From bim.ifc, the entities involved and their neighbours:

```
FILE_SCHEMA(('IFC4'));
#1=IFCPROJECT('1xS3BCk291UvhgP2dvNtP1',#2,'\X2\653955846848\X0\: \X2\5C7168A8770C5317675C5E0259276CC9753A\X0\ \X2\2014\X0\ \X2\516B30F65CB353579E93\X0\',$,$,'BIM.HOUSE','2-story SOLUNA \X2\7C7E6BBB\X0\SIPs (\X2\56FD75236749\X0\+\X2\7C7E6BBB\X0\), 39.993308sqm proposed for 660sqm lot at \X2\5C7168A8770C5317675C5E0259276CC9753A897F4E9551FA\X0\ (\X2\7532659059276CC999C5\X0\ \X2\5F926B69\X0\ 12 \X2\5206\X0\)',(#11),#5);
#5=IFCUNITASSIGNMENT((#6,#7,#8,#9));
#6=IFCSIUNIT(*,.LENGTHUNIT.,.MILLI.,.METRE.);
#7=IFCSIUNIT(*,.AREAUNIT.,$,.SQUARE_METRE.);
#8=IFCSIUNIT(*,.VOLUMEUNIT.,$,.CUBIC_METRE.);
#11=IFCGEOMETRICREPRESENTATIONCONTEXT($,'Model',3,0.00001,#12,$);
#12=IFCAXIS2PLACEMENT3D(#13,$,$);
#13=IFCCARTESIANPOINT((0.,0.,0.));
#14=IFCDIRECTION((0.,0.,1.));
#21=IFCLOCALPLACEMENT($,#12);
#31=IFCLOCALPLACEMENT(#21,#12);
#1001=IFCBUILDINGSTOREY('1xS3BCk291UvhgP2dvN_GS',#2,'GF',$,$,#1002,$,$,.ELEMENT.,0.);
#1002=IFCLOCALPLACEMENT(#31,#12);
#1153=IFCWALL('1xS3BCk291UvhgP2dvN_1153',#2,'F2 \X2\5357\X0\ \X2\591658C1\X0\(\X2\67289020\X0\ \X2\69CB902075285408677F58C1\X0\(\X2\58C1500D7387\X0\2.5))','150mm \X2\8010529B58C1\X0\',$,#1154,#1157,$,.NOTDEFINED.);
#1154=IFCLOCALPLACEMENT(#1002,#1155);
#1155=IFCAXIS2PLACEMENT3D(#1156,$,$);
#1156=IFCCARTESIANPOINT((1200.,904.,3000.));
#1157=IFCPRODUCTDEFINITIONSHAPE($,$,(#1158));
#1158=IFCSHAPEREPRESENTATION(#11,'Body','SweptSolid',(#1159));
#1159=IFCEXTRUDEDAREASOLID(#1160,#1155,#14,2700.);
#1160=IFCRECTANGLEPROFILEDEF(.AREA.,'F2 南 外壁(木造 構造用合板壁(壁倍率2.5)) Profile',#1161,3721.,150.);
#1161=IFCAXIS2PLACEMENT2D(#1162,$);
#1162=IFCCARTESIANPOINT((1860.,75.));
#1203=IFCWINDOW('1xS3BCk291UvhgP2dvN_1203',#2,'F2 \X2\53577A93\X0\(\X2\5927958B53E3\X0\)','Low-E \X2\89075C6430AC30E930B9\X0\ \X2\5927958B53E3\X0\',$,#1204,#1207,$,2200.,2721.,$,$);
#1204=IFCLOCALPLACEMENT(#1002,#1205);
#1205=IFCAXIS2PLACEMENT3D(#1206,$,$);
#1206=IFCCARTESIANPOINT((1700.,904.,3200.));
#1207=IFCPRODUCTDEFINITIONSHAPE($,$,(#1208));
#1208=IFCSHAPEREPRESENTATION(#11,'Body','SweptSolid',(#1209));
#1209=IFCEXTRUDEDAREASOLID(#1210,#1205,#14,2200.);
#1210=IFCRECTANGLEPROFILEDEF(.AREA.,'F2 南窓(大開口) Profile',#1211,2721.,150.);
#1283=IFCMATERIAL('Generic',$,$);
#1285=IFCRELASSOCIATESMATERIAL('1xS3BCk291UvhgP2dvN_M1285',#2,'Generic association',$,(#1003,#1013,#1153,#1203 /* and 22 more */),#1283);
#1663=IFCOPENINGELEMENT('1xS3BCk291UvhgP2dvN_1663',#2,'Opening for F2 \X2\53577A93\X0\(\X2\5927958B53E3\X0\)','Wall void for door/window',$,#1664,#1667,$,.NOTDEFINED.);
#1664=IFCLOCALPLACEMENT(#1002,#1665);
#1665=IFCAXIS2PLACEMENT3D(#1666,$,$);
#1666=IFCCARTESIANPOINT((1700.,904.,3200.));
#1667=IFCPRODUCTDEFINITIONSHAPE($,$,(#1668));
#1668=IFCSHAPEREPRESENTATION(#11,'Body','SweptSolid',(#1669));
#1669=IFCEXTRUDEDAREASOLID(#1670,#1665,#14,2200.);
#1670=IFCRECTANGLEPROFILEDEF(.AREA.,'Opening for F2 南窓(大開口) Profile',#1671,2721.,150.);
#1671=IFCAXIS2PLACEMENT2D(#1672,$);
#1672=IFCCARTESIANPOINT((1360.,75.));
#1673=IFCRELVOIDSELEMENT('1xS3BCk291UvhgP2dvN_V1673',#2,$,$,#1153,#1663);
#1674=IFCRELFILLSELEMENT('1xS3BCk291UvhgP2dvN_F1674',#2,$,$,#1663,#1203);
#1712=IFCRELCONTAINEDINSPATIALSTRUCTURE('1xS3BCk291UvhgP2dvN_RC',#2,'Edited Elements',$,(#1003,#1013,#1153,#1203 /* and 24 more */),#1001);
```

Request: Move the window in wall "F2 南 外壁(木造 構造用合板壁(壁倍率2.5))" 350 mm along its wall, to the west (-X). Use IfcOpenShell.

```python
import ifcopenshell
import ifcopenshell.api.geometry
import ifcopenshell.util.placement

model = ifcopenshell.open("bim.ifc")

window = model.by_guid("1xS3BCk291UvhgP2dvN_1203")
opening = window.FillsVoids[0].RelatingOpeningElement
wall = opening.VoidsElements[0].RelatingBuildingElement

wall_matrix = ifcopenshell.util.placement.get_local_placement(wall.ObjectPlacement)
shift = wall_matrix[:3, 0] * -350.0
before = ifcopenshell.util.placement.get_local_placement(window.ObjectPlacement)[:3, 3].copy()

# The window is not placed relative to its opening, so move both.
for product in (opening, window):
    matrix = ifcopenshell.util.placement.get_local_placement(product.ObjectPlacement)
    matrix[:3, 3] += shift
    ifcopenshell.api.geometry.edit_object_placement(model, product=product, matrix=matrix, is_si=False)

after = ifcopenshell.util.placement.get_local_placement(window.ObjectPlacement)[:3, 3]
print("window moved by", (after - before).round(3) + 0.0)

model.write("bim_updated.ifc")
```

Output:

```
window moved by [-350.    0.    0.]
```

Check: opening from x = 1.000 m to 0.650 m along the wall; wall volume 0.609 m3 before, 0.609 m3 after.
